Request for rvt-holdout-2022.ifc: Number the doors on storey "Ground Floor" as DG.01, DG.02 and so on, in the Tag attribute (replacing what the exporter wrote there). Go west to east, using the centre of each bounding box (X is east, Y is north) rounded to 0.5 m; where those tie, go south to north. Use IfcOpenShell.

First a look at what the model holds.

```python
import ifcopenshell
import ifcopenshell.util.element
import ifcopenshell.util.placement

model = ifcopenshell.open("rvt-holdout-2022.ifc")
print(model.schema)
storey = next(s for s in model.by_type("IfcBuildingStorey") if s.Name == "Ground Floor")
doors = [e for e in ifcopenshell.util.element.get_decomposition(storey) if e.is_a("IfcDoor")]
for e in sorted(doors, key=lambda e: e.id()):
    origin = ifcopenshell.util.placement.get_local_placement(e.ObjectPlacement)[:3, 3]
    print(e.id(), e.Tag, e.Name, origin.round(2) + 0.0, sep=" | ")
```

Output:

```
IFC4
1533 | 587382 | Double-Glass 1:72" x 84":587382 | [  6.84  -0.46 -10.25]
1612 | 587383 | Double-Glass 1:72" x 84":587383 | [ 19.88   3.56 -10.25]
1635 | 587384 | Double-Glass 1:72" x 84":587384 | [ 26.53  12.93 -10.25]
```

```python
import ifcopenshell
import ifcopenshell.geom
import ifcopenshell.util.element
import ifcopenshell.util.shape

model = ifcopenshell.open("rvt-holdout-2022.ifc")
settings = ifcopenshell.geom.settings()
settings.set("use-world-coords", True)


def centre(element):
    shape = ifcopenshell.geom.create_shape(settings, element)
    return ifcopenshell.util.shape.get_bbox_centroid(shape.geometry)


storey = next(s for s in model.by_type("IfcBuildingStorey") if s.Name == "Ground Floor")
doors = [e for e in ifcopenshell.util.element.get_decomposition(storey) if e.is_a("IfcDoor")]

# Insertion points can sit at a corner or the storey origin, so sort by the geometry (in metres).
centres = {e: centre(e) for e in doors}
doors.sort(key=lambda e: (round(centres[e][0] / 0.5), centres[e][1]))

for i, e in enumerate(doors, start=1):
    number = f"DG.{i:02d}"
    e.Tag = number
    print(e.id(), number)

model.write("rvt-holdout-2022_edited.ifc")
```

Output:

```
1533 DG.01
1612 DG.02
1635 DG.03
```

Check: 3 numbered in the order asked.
